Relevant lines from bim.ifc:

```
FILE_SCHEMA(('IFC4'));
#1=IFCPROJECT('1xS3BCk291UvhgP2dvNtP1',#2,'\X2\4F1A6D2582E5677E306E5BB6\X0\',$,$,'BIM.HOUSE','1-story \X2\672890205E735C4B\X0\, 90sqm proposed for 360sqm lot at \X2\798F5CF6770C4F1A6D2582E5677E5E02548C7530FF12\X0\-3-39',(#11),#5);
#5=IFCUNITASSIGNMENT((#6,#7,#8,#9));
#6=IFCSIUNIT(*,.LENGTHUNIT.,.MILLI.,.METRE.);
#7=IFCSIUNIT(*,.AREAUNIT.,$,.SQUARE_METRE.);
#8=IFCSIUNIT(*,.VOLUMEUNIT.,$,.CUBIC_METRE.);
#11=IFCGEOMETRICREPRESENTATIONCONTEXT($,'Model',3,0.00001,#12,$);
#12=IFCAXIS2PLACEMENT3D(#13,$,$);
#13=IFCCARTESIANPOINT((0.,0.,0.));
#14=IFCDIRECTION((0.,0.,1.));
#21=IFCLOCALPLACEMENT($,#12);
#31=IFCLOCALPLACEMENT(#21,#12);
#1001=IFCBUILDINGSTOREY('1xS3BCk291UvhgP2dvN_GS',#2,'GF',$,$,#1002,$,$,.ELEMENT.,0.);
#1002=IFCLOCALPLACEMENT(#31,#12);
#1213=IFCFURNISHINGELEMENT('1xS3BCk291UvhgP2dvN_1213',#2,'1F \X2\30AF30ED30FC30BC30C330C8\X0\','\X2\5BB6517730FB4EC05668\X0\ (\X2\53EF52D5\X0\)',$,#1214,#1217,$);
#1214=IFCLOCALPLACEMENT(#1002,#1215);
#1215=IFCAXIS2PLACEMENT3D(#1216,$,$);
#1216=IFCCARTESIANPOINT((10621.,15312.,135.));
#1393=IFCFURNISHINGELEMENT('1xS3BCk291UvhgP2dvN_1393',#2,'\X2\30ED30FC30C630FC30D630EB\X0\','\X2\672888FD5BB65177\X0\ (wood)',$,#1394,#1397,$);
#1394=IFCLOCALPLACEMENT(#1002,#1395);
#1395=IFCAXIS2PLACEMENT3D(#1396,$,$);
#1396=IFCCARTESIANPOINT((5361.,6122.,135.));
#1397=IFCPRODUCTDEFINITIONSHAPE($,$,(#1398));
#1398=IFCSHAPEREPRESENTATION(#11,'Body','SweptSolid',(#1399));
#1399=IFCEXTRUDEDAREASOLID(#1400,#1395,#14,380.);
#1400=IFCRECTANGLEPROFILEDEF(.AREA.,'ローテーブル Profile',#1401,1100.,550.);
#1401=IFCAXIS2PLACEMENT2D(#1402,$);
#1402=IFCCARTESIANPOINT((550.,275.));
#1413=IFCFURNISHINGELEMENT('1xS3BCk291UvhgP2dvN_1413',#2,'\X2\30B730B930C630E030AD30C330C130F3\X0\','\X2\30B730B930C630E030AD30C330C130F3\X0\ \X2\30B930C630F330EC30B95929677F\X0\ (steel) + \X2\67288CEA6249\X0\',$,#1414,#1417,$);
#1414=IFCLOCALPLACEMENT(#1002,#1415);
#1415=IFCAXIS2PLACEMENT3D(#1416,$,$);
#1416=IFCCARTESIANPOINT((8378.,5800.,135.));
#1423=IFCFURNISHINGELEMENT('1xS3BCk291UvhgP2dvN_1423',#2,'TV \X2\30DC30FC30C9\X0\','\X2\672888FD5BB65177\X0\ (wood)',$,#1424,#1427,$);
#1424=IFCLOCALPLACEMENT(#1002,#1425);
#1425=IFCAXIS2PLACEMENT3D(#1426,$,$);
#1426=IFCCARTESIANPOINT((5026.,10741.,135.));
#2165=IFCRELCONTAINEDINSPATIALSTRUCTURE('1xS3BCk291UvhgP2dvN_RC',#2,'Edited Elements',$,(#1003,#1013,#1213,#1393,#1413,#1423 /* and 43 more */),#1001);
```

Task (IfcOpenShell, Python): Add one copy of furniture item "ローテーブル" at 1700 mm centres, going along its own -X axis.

```python
import ifcopenshell
import ifcopenshell.api.geometry
import ifcopenshell.api.root
import ifcopenshell.util.element
import ifcopenshell.util.placement
import ifcopenshell.util.unit

model = ifcopenshell.open("bim.ifc")
unit_scale = ifcopenshell.util.unit.calculate_unit_scale(model)


def reuse_history(source, copy):
    """copy_class also copies each property set's owner history, people and application; keep the originals."""
    for rel in copy.IsDefinedBy:
        if rel.is_a("IfcRelDefinesByProperties") and (history := rel.RelatingPropertyDefinition.OwnerHistory):
            rel.RelatingPropertyDefinition.OwnerHistory = source.OwnerHistory
            ifcopenshell.util.element.remove_deep2(model, history)


source = model.by_guid("1xS3BCk291UvhgP2dvN_1393")
base = ifcopenshell.util.placement.get_local_placement(source.ObjectPlacement)
step = -base[:3, 0] * 1.7 / unit_scale

for i in range(1, 2):
    copy = ifcopenshell.api.root.copy_class(model, product=source)
    copy.Representation = ifcopenshell.util.element.copy_deep(
        model, source.Representation, exclude=["IfcGeometricRepresentationContext", "IfcRepresentationMap"]
    )
    reuse_history(source, copy)
    matrix = base.copy()
    matrix[:3, 3] += i * step
    print("added at", matrix[:3, 3].round(3) + 0.0)
    ifcopenshell.api.geometry.edit_object_placement(model, product=copy, matrix=matrix, is_si=False)

model.write("bim-out.ifc")
```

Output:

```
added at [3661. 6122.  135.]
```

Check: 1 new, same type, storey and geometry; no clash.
